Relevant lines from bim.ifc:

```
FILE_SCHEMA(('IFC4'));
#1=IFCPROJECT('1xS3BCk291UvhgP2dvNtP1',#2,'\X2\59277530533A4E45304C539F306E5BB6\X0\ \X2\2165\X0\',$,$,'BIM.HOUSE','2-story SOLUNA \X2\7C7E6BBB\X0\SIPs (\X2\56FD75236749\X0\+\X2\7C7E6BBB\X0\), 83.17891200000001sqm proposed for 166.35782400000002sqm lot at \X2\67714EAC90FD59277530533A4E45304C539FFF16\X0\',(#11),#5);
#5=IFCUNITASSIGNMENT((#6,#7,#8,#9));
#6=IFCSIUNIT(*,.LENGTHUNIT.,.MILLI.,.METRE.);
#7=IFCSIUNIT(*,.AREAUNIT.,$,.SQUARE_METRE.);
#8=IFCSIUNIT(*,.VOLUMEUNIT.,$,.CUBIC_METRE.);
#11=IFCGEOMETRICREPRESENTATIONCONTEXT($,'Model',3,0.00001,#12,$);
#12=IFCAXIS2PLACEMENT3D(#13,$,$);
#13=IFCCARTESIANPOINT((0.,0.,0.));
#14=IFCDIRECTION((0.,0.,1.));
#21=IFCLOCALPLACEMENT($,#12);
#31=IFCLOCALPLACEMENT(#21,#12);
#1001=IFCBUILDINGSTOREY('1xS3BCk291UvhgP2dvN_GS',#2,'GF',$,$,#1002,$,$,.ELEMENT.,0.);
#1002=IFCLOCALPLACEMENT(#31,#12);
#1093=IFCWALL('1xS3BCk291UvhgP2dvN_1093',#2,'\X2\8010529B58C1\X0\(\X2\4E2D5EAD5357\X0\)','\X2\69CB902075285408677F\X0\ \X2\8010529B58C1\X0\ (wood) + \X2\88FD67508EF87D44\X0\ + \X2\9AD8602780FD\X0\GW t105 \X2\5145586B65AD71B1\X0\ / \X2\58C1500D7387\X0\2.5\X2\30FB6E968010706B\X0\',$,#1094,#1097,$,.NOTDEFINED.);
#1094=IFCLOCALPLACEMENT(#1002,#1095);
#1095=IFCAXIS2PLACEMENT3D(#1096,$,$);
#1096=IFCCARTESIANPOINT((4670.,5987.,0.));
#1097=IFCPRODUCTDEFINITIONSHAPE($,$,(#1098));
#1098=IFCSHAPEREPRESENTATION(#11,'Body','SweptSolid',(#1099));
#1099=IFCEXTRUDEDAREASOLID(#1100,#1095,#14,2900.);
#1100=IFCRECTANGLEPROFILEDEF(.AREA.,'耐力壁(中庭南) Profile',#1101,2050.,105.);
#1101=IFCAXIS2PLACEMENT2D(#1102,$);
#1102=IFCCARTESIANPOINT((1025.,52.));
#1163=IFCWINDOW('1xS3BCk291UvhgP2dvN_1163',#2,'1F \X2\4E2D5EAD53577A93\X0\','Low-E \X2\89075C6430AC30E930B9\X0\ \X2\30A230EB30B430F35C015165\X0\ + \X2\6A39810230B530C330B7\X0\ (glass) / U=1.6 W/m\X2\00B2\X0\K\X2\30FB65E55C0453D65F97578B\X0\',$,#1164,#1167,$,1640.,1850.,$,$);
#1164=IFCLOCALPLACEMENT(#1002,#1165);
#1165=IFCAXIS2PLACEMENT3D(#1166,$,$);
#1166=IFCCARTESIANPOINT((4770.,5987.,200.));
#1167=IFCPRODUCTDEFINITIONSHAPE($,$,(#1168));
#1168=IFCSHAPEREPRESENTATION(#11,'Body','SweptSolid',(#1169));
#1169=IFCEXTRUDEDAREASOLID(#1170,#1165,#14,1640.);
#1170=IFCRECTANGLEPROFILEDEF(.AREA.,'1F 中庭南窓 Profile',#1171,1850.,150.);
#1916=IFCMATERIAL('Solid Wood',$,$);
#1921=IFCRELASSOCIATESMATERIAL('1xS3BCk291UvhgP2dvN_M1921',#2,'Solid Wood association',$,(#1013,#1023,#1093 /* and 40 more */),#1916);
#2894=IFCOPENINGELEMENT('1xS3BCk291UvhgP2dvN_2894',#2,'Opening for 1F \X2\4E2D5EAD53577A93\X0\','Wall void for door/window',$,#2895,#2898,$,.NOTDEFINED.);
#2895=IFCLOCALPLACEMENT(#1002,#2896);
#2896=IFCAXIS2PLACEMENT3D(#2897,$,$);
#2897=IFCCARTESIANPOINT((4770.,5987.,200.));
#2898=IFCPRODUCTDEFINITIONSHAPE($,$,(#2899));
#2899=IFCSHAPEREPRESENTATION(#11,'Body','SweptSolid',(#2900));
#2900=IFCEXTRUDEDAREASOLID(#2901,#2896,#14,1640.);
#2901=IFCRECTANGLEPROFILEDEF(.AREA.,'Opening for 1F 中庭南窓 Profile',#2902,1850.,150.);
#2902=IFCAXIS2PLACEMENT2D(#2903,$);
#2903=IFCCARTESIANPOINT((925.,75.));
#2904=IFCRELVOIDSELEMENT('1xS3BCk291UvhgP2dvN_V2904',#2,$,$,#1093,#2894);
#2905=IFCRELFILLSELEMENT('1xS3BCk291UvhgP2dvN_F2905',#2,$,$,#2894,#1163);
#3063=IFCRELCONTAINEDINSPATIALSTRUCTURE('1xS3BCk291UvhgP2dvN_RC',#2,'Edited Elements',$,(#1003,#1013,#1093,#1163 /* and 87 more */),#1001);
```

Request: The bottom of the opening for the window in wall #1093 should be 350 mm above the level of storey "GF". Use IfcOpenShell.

```python
import numpy as np
import ifcopenshell
import ifcopenshell.api.geometry
import ifcopenshell.geom
import ifcopenshell.util.element
import ifcopenshell.util.placement
import ifcopenshell.util.shape
import ifcopenshell.util.unit

model = ifcopenshell.open("bim.ifc")
unit_scale = ifcopenshell.util.unit.calculate_unit_scale(model)

window = model.by_id(1163)
opening = window.FillsVoids[0].RelatingOpeningElement
storey = ifcopenshell.util.element.get_container(window, ifc_class="IfcBuildingStorey")
level = ifcopenshell.util.placement.get_local_placement(storey.ObjectPlacement)[2, 3]

# The opening's origin need not be at the sill, so measure its lowest point.
shape = ifcopenshell.geom.create_shape(ifcopenshell.geom.settings(), opening)
bottom = ifcopenshell.util.shape.get_shape_bottom_elevation(shape, shape.geometry) / unit_scale
dz = level + 0.35 / unit_scale - bottom

shift = np.array([0.0, 0.0, dz])
# The window is not placed relative to its opening, so move both.
for product in (opening, window):
    matrix = ifcopenshell.util.placement.get_local_placement(product.ObjectPlacement)
    matrix[:3, 3] += shift
    ifcopenshell.api.geometry.edit_object_placement(model, product=product, matrix=matrix, is_si=False)

print(f"moved by {dz * unit_scale:+.3f} m")

model.write("bim_rev.ifc")
```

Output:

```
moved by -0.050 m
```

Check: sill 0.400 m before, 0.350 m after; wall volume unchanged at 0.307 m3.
